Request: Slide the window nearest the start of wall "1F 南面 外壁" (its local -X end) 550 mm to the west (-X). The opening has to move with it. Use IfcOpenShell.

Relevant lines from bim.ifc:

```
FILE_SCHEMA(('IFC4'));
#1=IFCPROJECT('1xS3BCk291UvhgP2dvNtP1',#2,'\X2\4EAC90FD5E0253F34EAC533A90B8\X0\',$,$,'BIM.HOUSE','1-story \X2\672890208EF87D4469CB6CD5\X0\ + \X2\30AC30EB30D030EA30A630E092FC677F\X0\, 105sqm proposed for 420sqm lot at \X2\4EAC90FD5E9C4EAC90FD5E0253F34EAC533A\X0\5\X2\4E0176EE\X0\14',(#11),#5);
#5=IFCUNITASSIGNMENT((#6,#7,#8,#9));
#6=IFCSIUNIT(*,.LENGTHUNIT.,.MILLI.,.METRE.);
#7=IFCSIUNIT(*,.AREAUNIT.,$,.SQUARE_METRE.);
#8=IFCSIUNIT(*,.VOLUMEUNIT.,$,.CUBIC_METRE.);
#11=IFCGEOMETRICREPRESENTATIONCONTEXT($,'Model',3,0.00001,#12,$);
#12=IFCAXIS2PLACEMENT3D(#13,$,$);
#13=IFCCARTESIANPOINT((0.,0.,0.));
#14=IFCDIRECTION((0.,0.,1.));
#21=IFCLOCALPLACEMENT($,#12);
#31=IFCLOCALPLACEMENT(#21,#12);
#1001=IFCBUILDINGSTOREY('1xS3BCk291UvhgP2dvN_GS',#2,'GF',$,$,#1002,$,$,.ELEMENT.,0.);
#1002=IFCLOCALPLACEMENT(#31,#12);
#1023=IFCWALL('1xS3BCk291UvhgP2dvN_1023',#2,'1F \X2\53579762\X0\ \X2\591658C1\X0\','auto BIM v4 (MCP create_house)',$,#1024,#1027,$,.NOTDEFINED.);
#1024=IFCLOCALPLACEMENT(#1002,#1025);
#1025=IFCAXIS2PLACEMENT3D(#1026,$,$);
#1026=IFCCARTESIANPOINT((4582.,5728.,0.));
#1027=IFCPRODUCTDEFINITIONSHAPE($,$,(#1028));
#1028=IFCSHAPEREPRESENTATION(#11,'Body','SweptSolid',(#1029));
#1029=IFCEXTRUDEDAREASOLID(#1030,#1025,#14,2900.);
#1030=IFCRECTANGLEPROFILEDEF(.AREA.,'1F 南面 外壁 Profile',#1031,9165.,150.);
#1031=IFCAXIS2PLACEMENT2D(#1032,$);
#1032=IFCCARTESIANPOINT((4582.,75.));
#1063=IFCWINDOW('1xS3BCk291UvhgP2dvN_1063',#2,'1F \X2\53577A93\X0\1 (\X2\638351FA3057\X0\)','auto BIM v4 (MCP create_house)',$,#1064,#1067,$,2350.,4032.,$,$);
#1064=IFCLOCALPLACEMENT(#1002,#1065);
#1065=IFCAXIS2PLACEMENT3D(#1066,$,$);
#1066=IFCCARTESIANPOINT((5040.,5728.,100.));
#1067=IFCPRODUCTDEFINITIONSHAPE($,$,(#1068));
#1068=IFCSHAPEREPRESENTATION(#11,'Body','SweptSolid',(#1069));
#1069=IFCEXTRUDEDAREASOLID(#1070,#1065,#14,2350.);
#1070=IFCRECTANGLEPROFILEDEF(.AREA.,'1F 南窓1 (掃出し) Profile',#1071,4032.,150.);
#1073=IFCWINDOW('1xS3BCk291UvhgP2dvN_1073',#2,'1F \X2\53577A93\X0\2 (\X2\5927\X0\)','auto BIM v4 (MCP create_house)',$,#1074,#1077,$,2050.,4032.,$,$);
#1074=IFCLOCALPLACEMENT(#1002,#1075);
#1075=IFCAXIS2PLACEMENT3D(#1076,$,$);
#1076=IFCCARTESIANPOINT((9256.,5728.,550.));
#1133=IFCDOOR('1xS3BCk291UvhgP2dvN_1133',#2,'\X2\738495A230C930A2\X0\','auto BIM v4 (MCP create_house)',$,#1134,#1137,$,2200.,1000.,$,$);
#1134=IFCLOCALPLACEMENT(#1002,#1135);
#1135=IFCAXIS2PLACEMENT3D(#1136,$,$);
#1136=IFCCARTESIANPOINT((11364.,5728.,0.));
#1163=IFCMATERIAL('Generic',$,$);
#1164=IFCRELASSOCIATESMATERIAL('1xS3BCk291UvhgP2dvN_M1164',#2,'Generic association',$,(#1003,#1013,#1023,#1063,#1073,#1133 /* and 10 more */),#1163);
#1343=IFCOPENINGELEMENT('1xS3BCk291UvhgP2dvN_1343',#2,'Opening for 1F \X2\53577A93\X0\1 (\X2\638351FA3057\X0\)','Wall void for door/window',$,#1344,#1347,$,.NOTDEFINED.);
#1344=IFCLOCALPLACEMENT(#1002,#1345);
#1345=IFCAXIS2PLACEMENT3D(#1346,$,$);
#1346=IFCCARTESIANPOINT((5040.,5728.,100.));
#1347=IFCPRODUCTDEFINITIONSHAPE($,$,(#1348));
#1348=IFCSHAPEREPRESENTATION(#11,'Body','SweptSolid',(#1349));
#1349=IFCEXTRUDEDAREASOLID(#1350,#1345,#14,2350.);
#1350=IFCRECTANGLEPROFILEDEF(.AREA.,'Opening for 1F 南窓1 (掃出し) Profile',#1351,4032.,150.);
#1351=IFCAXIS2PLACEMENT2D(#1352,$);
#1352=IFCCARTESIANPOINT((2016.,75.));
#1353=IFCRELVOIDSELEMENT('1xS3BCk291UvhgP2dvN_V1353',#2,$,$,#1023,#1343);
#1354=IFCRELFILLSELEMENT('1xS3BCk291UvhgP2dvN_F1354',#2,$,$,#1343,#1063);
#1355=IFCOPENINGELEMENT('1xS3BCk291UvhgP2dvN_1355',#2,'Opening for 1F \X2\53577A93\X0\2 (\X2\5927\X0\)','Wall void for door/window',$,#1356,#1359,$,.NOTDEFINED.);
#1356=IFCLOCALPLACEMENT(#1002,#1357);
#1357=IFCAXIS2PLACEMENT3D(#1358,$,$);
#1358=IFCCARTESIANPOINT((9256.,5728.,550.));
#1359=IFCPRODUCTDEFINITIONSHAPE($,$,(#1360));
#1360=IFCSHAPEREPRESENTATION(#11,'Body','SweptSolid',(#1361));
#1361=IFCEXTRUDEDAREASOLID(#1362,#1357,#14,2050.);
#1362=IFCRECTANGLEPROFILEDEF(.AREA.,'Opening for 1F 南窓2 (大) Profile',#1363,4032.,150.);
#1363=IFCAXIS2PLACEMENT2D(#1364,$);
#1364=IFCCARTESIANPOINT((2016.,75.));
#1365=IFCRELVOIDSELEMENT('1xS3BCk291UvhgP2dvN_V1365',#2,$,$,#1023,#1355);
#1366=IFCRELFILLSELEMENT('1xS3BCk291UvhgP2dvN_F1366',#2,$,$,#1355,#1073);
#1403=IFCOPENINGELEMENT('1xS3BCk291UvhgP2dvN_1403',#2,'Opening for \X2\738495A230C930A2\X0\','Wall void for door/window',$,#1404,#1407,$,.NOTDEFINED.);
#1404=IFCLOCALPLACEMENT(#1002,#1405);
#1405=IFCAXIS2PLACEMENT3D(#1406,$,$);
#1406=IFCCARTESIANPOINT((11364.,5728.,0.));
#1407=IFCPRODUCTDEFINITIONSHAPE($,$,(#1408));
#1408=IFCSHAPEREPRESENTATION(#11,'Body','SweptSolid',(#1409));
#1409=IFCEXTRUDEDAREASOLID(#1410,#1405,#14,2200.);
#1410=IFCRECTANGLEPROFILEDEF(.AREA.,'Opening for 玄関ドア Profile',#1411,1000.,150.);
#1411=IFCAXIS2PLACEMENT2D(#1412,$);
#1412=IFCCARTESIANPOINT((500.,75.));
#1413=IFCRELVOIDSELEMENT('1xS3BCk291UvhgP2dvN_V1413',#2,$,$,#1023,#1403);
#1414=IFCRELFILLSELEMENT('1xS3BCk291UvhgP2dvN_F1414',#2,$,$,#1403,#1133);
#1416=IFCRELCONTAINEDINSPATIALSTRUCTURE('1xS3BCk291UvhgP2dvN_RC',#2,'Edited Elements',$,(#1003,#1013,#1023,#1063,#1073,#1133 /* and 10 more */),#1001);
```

```python
import ifcopenshell
import ifcopenshell.api.geometry
import ifcopenshell.util.placement
import ifcopenshell.util.unit

model = ifcopenshell.open("bim.ifc")
unit_scale = ifcopenshell.util.unit.calculate_unit_scale(model)

window = model.by_guid("1xS3BCk291UvhgP2dvN_1063")
opening = window.FillsVoids[0].RelatingOpeningElement
wall = opening.VoidsElements[0].RelatingBuildingElement

wall_matrix = ifcopenshell.util.placement.get_local_placement(wall.ObjectPlacement)
shift = wall_matrix[:3, 0] * -0.55 / unit_scale
before = ifcopenshell.util.placement.get_local_placement(window.ObjectPlacement)[:3, 3].copy()

# The window is not placed relative to its opening, so move both.
for product in (opening, window):
    matrix = ifcopenshell.util.placement.get_local_placement(product.ObjectPlacement)
    matrix[:3, 3] += shift
    ifcopenshell.api.geometry.edit_object_placement(model, product=product, matrix=matrix, is_si=False)

after = ifcopenshell.util.placement.get_local_placement(window.ObjectPlacement)[:3, 3]
print("window moved by", (after - before).round(3) + 0.0)

model.write("bim-out.ifc")
```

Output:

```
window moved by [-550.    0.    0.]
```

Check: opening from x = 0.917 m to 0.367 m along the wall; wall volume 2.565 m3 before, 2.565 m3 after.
